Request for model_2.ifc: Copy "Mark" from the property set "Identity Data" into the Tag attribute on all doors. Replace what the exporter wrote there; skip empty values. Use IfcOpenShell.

First a look at what the model holds.

```python
import ifcopenshell
import ifcopenshell.util.element

model = ifcopenshell.open("model_2.ifc")
print(model.schema)
doors = model.by_type("IfcDoor")
print(len(doors), "doors")
for e in doors[:8]:
    source = ifcopenshell.util.element.get_pset(e, "Identity Data", "Mark")
    target = e.Tag
    print(e.id(), repr(source), repr(target), sep=" | ")
```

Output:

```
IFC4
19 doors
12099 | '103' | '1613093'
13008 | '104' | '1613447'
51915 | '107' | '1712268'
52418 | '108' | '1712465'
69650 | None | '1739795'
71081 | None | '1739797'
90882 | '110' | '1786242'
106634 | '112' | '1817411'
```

```python
import ifcopenshell
import ifcopenshell.util.element

model = ifcopenshell.open("model_2.ifc")

count = 0
for e in model.by_type("IfcDoor"):
    value = ifcopenshell.util.element.get_pset(e, "Identity Data", "Mark")
    current = e.Tag
    if not value or not value.strip() or current == value:
        continue
    e.Tag = value
    count += 1

print(count, "doors updated")

model.write("model_2_updated.ifc")
```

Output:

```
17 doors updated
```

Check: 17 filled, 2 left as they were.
